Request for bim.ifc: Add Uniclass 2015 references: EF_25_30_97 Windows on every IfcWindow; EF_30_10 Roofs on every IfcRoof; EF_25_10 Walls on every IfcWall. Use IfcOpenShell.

First a look at what the model holds.

```python
import ifcopenshell

model = ifcopenshell.open("bim.ifc")
print(model.schema)
print("classifications:", [c.Name for c in model.by_type("IfcClassification")])
for ifc_class in ("IfcDoor", "IfcRoof", "IfcStair", "IfcWall", "IfcWindow"):
    print(ifc_class, len(model.by_type(ifc_class)))
```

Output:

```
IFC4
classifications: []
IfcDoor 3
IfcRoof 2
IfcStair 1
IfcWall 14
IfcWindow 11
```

```python
import ifcopenshell
import ifcopenshell.api.classification

model = ifcopenshell.open("bim.ifc")

system = ifcopenshell.api.classification.add_classification(model, classification="Uniclass 2015")

codes = {
    "IfcWindow": ("EF_25_30_97", "Windows"),
    "IfcRoof": ("EF_30_10", "Roofs"),
    "IfcWall": ("EF_25_10", "Walls"),
}
for ifc_class, (code, name) in codes.items():
    products = model.by_type(ifc_class)
    ifcopenshell.api.classification.add_reference(
        model, products=products, classification=system, identification=code, name=name
    )
    print(code, len(products))

model.write("bim_edited.ifc")
```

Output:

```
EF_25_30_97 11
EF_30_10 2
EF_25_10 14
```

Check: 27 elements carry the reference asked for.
